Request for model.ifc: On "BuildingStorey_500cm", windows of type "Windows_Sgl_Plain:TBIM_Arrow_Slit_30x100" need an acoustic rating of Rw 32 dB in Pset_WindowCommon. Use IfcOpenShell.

First a look at what the model holds.

```python
import ifcopenshell
import ifcopenshell.util.element

model = ifcopenshell.open("model.ifc")
print(model.schema)
storey = next(s for s in model.by_type("IfcBuildingStorey") if s.Name == "BuildingStorey_500cm")
windows = [e for e in ifcopenshell.util.element.get_decomposition(storey) if e.is_a("IfcWindow")]
seen = {}
for e in windows:
    element_type = ifcopenshell.util.element.get_type(e)
    key = (element_type.Name if element_type != e and element_type else None, ifcopenshell.util.element.get_pset(e, "Pset_WindowCommon", "AcousticRating"))
    seen[key] = seen.get(key, 0) + 1
for (name, value), count in sorted(seen.items(), key=str):
    print(count, "x", name, "|", value)
```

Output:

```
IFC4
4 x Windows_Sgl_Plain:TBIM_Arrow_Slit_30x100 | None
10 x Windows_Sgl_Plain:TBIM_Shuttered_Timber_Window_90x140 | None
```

```python
import ifcopenshell
import ifcopenshell.api.pset
import ifcopenshell.util.element

model = ifcopenshell.open("model.ifc")

storey = next(s for s in model.by_type("IfcBuildingStorey") if s.Name == "BuildingStorey_500cm")
windows = [e for e in ifcopenshell.util.element.get_decomposition(storey) if e.is_a("IfcWindow")]

count = 0
for e in windows:
    element_type = ifcopenshell.util.element.get_type(e)
    if element_type in (None, e) or element_type.Name != "Windows_Sgl_Plain:TBIM_Arrow_Slit_30x100":
        continue
    # add_pset returns the element's existing set when there is one.
    pset = ifcopenshell.api.pset.add_pset(model, product=e, name="Pset_WindowCommon")
    ifcopenshell.api.pset.edit_pset(model, pset=pset, properties={"AcousticRating": "Rw 32 dB"})
    count += 1

print(count, "windows updated")

model.write("model_v2.ifc")
```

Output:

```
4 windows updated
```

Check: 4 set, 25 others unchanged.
